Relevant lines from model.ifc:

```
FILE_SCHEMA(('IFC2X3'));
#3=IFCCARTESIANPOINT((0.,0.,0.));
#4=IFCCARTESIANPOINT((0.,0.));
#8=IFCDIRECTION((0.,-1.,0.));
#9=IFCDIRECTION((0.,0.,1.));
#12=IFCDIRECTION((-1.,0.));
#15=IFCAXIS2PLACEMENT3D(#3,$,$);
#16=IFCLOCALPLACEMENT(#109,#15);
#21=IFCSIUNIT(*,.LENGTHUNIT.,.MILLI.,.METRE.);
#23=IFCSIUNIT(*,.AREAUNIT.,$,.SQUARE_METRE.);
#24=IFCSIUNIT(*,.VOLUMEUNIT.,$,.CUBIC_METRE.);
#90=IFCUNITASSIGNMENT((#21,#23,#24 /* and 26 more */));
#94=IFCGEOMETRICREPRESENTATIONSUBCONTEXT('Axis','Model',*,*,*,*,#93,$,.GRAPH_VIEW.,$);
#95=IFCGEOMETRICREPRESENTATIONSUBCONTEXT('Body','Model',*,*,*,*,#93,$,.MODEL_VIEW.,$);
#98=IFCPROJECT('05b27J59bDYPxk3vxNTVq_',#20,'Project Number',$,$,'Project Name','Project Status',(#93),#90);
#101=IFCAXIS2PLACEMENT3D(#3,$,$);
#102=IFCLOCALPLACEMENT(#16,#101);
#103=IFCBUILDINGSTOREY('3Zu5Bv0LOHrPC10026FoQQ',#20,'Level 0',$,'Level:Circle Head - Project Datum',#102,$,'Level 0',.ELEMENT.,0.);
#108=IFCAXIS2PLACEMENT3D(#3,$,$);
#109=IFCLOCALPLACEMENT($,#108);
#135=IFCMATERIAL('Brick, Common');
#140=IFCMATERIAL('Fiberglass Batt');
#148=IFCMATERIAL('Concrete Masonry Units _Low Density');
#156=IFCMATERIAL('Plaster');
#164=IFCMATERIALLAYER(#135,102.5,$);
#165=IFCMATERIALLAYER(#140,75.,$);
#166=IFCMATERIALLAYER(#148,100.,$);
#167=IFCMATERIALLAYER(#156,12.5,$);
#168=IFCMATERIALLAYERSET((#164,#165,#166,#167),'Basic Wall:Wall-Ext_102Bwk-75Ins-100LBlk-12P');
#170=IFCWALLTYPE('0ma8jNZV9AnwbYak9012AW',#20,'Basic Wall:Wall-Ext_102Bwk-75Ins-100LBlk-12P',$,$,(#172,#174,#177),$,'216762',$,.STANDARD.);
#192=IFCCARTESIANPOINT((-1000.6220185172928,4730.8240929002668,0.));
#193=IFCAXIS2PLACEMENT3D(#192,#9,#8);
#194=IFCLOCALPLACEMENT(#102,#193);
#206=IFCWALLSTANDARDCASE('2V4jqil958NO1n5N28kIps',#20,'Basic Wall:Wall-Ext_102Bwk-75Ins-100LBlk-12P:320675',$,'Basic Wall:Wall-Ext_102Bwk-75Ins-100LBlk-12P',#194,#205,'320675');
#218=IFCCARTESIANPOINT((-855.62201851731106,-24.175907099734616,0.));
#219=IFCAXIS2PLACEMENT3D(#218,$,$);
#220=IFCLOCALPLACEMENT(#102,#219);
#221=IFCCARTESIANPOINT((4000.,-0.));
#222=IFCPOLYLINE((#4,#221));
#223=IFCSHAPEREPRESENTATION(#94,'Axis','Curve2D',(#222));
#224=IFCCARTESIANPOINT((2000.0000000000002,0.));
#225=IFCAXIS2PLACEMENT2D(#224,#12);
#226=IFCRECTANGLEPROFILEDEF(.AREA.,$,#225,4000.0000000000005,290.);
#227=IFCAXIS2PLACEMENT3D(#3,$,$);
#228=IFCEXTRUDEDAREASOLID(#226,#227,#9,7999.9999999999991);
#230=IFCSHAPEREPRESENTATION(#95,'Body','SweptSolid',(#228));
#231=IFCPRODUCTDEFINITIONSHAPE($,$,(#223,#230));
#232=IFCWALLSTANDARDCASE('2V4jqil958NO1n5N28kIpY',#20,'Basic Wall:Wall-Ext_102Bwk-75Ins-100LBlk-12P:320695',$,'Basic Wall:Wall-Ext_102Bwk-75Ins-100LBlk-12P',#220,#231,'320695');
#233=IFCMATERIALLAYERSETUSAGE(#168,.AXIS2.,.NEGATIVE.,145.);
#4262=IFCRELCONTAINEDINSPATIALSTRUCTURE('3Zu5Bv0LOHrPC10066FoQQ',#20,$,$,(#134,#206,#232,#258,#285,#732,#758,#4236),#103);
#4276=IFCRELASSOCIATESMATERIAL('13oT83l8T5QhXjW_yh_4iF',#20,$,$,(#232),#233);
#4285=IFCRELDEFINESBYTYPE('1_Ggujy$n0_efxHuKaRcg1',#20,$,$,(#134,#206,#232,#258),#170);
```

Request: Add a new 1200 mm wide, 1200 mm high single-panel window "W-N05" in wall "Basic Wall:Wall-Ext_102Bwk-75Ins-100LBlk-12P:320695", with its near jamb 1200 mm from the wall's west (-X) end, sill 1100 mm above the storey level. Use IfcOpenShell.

```python
import numpy as np
import ifcopenshell
import ifcopenshell.api.feature
import ifcopenshell.api.geometry
import ifcopenshell.api.root
import ifcopenshell.api.spatial
import ifcopenshell.api.type
import ifcopenshell.geom
import ifcopenshell.util.element
import ifcopenshell.util.placement
import ifcopenshell.util.representation
import ifcopenshell.util.shape
import ifcopenshell.util.unit

model = ifcopenshell.open("model.ifc")
unit_scale = ifcopenshell.util.unit.calculate_unit_scale(model)
settings = ifcopenshell.geom.settings()


def volume(element):
    """Net volume in cubic metres, openings subtracted."""
    shape = ifcopenshell.geom.create_shape(settings, element)
    return ifcopenshell.util.shape.get_volume(shape.geometry)


wall = model.by_guid("2V4jqil958NO1n5N28kIpY")
storey = ifcopenshell.util.element.get_container(wall, ifc_class="IfcBuildingStorey")
context = ifcopenshell.util.representation.get_context(model, "Model", "Body", "MODEL_VIEW")
before = volume(wall)

width, height, from_end, sill = 1.2, 1.2, 1.2, 1.1  # metres

# The wall runs along its own X axis, and the end named is its -X end.
wall_shape = ifcopenshell.geom.create_shape(settings, wall)
x, y, z = ifcopenshell.util.shape.get_vertices(wall_shape.geometry).T
start = x.min() + from_end
face, thickness = float(y.min()), float(y.max() - y.min())
wall_matrix = ifcopenshell.util.placement.get_local_placement(wall.ObjectPlacement)
level = ifcopenshell.util.placement.get_local_placement(storey.ObjectPlacement)[2, 3]


def in_wall(x, y):
    """Placement at x, y metres in the wall's axes, at sill height."""
    matrix = wall_matrix.copy()
    matrix[:, 3] = wall_matrix @ np.array([x / unit_scale, y / unit_scale, 0.0, 1.0])
    matrix[2, 3] = level + sill / unit_scale
    return matrix


# Opening: a box that overshoots both wall faces by 50 mm.
opening = ifcopenshell.api.root.create_entity(model, ifc_class="IfcOpeningElement")
box = ifcopenshell.api.geometry.add_wall_representation(
    model, context=context, length=width, height=height, thickness=thickness + 0.1
)
ifcopenshell.api.geometry.assign_representation(model, product=opening, representation=box)
ifcopenshell.api.geometry.edit_object_placement(model, product=opening, matrix=in_wall(start, face - 0.05), is_si=False)
ifcopenshell.api.feature.add_feature(model, feature=opening, element=wall)

window = ifcopenshell.api.root.create_entity(model, ifc_class="IfcWindow", name="W-N05")
window.OverallWidth, window.OverallHeight = width / unit_scale, height / unit_scale
body = ifcopenshell.api.geometry.add_window_representation(
    model,
    context=context,
    overall_width=window.OverallWidth,
    overall_height=window.OverallHeight,
    partition_type="SINGLE_PANEL",
)
ifcopenshell.api.geometry.assign_representation(model, product=window, representation=body)
ifcopenshell.api.spatial.assign_container(model, products=[window], relating_structure=storey)
fills = ifcopenshell.api.feature.add_filling(model, opening=opening, element=window)
fills.OwnerHistory = window.OwnerHistory  # required in IFC2X3

# IFC2X3 keeps the operation on the window style.
style = ifcopenshell.api.root.create_entity(model, ifc_class="IfcWindowStyle", name="W-N05")
style.OperationType, style.ConstructionType = "SINGLE_PANEL", "NOTDEFINED"
style.ParameterTakesPrecedence = style.Sizeable = False
ifcopenshell.api.type.assign_type(model, related_objects=[window], relating_type=style)

# Centre the window in the wall's thickness.
ifcopenshell.api.geometry.edit_object_placement(model, product=window, matrix=in_wall(start, face), is_si=False)
window_shape = ifcopenshell.geom.create_shape(settings, window)
depth = ifcopenshell.util.shape.get_vertices(window_shape.geometry)[:, 1]
offset = face + thickness / 2 - (depth.min() + depth.max()) / 2
ifcopenshell.api.geometry.edit_object_placement(model, product=window, matrix=in_wall(start, offset), is_si=False)

after = volume(wall)

print(f"wall volume {before:.3f} -> {after:.3f} m3")

model.write("model_v2.ifc")
```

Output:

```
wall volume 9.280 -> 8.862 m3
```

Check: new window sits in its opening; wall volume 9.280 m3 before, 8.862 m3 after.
